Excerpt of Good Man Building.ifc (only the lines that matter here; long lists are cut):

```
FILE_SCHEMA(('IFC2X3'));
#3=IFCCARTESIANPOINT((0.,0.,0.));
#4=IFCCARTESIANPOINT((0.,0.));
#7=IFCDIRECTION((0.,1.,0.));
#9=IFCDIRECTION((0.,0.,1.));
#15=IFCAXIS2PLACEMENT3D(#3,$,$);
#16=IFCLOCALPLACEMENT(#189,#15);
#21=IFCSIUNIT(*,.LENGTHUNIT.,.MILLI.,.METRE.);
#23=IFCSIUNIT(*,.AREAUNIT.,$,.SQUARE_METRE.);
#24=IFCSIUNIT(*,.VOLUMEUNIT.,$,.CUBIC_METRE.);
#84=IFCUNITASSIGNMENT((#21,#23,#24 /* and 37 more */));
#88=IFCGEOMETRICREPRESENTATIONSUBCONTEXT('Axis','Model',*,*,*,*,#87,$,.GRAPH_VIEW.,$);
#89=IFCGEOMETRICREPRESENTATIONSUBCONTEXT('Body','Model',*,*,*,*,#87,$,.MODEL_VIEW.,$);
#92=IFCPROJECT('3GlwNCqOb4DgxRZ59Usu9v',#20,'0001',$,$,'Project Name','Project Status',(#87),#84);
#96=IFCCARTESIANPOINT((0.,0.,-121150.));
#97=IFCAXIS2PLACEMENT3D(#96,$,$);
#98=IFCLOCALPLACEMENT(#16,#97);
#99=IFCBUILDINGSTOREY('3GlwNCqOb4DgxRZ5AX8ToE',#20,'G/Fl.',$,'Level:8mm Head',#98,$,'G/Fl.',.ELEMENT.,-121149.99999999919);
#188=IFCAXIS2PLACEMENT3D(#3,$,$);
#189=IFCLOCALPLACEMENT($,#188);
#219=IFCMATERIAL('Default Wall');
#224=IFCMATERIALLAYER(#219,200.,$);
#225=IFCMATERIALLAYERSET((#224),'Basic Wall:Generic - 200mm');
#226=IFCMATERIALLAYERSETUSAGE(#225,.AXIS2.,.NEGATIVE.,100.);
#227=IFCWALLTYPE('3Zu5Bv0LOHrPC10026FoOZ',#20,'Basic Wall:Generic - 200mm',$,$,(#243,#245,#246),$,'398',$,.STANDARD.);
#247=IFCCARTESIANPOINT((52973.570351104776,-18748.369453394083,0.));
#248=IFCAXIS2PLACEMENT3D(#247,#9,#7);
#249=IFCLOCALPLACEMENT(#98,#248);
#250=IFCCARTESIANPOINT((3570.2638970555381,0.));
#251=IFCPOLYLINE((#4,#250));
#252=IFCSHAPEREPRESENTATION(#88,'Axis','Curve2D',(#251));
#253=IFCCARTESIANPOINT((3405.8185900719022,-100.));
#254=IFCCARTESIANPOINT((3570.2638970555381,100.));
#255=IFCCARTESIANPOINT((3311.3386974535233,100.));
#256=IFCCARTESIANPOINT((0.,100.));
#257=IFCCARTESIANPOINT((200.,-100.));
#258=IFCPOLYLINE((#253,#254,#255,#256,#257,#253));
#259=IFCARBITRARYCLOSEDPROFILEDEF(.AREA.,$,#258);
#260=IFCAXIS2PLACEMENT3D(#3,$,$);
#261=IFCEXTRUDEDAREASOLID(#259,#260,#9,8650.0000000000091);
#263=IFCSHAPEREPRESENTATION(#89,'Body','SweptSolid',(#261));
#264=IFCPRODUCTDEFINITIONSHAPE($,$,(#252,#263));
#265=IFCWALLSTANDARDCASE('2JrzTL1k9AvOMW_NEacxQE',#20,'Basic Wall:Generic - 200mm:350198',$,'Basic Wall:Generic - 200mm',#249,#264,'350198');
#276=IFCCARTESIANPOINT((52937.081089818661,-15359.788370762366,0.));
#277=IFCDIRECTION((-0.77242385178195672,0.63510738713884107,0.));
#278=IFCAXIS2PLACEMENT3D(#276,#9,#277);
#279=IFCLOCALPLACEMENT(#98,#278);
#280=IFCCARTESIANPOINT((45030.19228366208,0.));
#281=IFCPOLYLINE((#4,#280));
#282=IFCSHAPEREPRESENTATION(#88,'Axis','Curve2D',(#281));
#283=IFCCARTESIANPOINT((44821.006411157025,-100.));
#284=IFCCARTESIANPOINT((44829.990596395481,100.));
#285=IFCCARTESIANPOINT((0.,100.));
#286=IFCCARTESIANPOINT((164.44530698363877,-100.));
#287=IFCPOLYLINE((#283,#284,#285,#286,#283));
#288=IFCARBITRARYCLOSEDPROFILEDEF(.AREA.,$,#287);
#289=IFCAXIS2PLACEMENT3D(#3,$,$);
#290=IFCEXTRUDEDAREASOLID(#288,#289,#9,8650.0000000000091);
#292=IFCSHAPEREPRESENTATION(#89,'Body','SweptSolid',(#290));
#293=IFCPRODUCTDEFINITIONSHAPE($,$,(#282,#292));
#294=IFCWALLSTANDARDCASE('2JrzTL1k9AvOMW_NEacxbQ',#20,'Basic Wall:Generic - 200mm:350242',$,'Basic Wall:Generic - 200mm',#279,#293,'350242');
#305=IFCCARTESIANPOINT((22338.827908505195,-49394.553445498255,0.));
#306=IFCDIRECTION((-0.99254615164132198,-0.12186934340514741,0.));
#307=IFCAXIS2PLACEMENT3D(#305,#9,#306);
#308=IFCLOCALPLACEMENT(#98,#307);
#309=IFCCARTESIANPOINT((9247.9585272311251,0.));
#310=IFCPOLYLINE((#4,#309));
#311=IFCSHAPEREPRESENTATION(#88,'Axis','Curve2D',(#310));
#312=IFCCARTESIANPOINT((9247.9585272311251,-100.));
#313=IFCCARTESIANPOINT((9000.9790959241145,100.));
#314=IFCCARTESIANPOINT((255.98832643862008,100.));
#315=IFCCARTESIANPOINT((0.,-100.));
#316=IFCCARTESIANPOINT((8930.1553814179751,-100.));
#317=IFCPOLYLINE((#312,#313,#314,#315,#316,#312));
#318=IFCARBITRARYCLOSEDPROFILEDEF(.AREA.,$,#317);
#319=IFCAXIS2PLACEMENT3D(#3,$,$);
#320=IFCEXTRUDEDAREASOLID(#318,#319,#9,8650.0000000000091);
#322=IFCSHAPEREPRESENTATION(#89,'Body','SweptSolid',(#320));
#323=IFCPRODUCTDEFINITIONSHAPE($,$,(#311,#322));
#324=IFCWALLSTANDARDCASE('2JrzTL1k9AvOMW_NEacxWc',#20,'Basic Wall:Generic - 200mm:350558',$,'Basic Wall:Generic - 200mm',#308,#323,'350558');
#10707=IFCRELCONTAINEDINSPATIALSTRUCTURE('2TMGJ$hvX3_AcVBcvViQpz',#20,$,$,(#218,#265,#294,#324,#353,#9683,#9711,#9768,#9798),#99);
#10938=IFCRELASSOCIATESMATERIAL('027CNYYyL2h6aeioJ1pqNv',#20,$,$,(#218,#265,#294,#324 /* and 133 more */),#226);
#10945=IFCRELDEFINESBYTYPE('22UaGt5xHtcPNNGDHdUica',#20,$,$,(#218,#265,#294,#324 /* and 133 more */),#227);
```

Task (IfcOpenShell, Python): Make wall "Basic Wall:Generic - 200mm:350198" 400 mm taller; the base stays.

```python
import ifcopenshell
import ifcopenshell.geom
import ifcopenshell.util.representation
import ifcopenshell.util.shape
import ifcopenshell.util.unit

model = ifcopenshell.open("Good Man Building.ifc")
unit_scale = ifcopenshell.util.unit.calculate_unit_scale(model)
settings = ifcopenshell.geom.settings()


def volume(element):
    """Net volume in cubic metres, openings subtracted."""
    shape = ifcopenshell.geom.create_shape(settings, element)
    return ifcopenshell.util.shape.get_volume(shape.geometry)


wall = model.by_guid("2JrzTL1k9AvOMW_NEacxQE")
before = volume(wall)

body = ifcopenshell.util.representation.get_representation(wall, "Model", "Body")
solid = body.Items[0]
old_height = solid.Depth
solid.Depth += 0.4 / unit_scale
after = volume(wall)

print(f"height {old_height:g} -> {solid.Depth:g}, volume {before:.3f} -> {after:.3f} m3")

model.write("Good Man Building_updated.ifc")
```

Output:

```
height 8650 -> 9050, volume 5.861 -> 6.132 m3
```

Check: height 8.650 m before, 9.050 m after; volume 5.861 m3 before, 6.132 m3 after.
